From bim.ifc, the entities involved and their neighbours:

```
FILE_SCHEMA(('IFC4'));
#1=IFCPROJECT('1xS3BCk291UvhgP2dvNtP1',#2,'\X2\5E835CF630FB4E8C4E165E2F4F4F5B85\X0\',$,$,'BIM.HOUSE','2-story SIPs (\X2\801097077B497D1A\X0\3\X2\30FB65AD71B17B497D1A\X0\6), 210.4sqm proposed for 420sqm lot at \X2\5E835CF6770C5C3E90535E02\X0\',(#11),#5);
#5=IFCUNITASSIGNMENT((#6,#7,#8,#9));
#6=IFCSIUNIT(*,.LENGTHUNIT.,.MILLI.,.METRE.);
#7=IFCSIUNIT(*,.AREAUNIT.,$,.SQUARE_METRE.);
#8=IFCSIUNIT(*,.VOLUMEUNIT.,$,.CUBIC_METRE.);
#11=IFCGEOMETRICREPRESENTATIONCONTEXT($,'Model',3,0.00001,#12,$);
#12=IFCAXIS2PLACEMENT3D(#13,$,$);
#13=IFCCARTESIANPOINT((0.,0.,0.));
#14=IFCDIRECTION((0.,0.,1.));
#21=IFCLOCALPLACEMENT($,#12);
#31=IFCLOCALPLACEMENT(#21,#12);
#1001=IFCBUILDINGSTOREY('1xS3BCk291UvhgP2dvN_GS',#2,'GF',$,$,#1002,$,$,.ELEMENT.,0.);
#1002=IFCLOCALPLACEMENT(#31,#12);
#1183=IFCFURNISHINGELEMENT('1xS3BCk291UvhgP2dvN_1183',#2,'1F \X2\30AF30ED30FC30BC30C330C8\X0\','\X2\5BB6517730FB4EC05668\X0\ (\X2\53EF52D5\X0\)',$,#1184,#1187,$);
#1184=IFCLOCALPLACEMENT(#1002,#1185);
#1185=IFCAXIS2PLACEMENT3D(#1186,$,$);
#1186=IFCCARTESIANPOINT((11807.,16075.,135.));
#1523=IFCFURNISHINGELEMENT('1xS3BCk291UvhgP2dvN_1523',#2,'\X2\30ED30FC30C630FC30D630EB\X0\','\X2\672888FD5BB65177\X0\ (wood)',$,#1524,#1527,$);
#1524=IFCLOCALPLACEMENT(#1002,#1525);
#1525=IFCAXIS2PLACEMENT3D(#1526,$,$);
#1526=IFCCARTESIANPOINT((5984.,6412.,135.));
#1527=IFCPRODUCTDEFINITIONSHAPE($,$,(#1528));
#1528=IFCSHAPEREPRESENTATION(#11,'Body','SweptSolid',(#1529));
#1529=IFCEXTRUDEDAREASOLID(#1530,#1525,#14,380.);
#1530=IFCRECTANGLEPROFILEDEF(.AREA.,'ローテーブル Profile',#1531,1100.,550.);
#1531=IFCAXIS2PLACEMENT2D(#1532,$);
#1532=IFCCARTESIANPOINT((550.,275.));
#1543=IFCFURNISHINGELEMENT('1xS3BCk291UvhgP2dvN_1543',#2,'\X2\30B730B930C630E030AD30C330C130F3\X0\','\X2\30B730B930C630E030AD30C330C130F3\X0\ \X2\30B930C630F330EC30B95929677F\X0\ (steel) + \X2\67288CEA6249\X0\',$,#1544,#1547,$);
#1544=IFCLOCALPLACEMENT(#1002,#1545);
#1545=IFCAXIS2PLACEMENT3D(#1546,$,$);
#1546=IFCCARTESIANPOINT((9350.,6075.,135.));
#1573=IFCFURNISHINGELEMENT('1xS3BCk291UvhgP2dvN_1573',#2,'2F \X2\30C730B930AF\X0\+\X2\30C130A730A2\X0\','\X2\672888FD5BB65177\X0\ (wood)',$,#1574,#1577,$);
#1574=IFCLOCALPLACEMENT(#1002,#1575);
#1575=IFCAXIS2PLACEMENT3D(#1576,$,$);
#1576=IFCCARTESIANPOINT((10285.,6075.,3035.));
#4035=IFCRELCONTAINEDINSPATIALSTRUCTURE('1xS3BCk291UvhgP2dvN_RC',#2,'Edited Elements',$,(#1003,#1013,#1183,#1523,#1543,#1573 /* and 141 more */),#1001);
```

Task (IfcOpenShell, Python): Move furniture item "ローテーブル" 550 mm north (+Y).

```python
import ifcopenshell
import ifcopenshell.api.geometry
import ifcopenshell.util.placement

model = ifcopenshell.open("bim.ifc")

item = model.by_guid("1xS3BCk291UvhgP2dvN_1523")
matrix = ifcopenshell.util.placement.get_local_placement(item.ObjectPlacement)
matrix[1, 3] += 550.0
ifcopenshell.api.geometry.edit_object_placement(model, product=item, matrix=matrix, is_si=False)

print(ifcopenshell.util.placement.get_local_placement(item.ObjectPlacement).round(3) + 0.0)

model.write("bim-out.ifc")
```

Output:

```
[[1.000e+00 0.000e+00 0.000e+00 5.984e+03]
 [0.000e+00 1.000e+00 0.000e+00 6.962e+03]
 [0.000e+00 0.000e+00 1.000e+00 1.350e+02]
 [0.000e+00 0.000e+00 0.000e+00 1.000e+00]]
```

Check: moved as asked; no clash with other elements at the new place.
